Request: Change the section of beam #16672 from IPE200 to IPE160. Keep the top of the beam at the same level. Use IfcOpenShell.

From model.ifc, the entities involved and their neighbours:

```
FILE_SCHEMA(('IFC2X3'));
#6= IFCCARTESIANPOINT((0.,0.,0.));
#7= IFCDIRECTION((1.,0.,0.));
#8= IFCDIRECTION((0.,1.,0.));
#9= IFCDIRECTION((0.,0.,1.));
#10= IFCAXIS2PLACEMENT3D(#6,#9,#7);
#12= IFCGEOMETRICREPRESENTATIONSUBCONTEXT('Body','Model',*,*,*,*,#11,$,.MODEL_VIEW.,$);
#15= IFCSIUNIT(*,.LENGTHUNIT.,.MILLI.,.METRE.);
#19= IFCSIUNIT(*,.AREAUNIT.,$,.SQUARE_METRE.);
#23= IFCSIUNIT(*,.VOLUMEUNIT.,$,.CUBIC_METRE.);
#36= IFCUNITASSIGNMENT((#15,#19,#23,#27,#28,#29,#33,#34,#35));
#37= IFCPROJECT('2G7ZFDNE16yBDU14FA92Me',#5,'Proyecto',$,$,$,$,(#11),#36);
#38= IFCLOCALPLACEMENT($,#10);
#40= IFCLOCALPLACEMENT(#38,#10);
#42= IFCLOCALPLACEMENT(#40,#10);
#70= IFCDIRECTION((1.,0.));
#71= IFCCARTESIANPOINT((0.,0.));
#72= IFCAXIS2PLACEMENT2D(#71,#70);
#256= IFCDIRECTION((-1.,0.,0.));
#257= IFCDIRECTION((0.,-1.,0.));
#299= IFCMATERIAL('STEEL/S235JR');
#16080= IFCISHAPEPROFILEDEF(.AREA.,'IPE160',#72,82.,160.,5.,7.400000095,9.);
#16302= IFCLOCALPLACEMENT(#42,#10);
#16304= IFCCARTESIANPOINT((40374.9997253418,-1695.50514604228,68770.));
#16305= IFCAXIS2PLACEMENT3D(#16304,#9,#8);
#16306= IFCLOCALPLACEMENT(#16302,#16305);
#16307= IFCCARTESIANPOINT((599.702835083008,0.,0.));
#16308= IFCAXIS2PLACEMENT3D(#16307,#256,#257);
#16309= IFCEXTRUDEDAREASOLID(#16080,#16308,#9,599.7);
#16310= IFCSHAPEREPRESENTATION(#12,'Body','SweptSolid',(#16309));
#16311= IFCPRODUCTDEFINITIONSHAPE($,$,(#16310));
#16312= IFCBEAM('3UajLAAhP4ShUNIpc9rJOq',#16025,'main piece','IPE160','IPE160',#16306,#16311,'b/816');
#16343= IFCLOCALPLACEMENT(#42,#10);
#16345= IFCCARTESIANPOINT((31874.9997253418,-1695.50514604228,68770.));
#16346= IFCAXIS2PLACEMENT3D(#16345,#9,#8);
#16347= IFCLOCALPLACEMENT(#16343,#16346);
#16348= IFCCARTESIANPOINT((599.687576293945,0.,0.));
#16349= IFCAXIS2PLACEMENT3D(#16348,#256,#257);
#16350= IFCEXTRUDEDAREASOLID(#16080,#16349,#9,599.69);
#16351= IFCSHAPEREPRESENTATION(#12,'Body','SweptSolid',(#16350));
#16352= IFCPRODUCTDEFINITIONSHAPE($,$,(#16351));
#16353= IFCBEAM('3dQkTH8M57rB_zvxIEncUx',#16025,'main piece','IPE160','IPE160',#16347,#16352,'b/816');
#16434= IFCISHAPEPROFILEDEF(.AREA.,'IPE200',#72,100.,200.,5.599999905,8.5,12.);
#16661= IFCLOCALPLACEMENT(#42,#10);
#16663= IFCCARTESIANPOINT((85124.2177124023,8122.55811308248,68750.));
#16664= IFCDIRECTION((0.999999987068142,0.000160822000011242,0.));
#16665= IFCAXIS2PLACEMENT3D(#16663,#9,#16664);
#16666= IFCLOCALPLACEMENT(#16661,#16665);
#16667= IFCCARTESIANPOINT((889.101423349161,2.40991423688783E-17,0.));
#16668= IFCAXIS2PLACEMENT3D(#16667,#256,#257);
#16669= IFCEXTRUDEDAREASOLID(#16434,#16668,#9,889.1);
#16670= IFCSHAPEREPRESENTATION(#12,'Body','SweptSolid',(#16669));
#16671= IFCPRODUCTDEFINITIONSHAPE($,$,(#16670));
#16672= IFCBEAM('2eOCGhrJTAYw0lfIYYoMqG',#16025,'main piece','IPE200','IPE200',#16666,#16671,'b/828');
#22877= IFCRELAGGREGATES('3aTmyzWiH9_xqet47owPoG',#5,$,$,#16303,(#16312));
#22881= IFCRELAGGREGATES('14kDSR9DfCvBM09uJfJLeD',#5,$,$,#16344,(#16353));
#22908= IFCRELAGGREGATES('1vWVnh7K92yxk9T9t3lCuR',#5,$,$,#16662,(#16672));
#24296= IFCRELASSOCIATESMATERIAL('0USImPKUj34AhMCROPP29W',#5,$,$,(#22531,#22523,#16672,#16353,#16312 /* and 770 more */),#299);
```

```python
import ifcopenshell
import ifcopenshell.util.element
import ifcopenshell.util.representation

model = ifcopenshell.open("model.ifc")

member = model.by_guid("2eOCGhrJTAYw0lfIYYoMqG")
source = next(p for p in model.by_type("IfcIShapeProfileDef") if p.ProfileName == "IPE160")

body = ifcopenshell.util.representation.get_representation(member, "Model", "Body")
solid = body.Items[0]
old_profile = solid.SweptArea

# Copy the section's sizes but keep this member's own profile position.
profile = ifcopenshell.util.element.copy(model, source)
# Profiles are centred, so shift by half the change in depth to hold the top.
shift = (old_profile.OverallDepth - profile.OverallDepth) / 2
x, y = old_profile.Position.Location.Coordinates
up = (0.0, 1.0)  # upwards, in the solid's own plane
location = model.createIfcCartesianPoint((x + up[0] * shift, y + up[1] * shift))
profile.Position = model.createIfcAxis2Placement2D(location, old_profile.Position.RefDirection)
solid.SweptArea = profile
if not model.get_total_inverses(old_profile):
    ifcopenshell.util.element.remove_deep2(model, old_profile)
member.Description = member.Description.replace("IPE200", "IPE160")
member.ObjectType = member.ObjectType.replace("IPE200", "IPE160")

print(solid.SweptArea)

model.write("model-out.ifc")
```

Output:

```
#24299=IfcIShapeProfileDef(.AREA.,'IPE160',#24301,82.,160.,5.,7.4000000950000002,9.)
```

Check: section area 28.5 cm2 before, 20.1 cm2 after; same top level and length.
